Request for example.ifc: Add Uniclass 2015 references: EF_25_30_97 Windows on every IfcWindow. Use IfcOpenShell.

First a look at what the model holds.

```python
import ifcopenshell

model = ifcopenshell.open("example.ifc")
print(model.schema)
print("classifications:", [c.Name for c in model.by_type("IfcClassification")])
for ifc_class in ("IfcDoor", "IfcRoof", "IfcStair", "IfcWall", "IfcWindow"):
    print(ifc_class, len(model.by_type(ifc_class)))
```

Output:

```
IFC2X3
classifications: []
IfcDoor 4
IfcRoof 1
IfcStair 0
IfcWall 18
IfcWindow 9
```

```python
import ifcopenshell
import ifcopenshell.api.classification

model = ifcopenshell.open("example.ifc")

# IFC2X3 requires Source and Edition and has no link from the project to the system.
system = model.create_entity("IfcClassification", Source="NBS", Edition="2015", Name="Uniclass 2015")

codes = {
    "IfcWindow": ("EF_25_30_97", "Windows"),
}
for ifc_class, (code, name) in codes.items():
    products = model.by_type(ifc_class)
    ifcopenshell.api.classification.add_reference(
        model, products=products, classification=system, identification=code, name=name
    )
    print(code, len(products))

model.write("example_rev.ifc")
```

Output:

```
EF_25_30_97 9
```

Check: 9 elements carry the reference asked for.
